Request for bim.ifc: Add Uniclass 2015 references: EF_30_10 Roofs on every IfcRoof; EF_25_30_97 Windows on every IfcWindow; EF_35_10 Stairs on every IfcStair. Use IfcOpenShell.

First a look at what the model holds.

```python
import ifcopenshell

model = ifcopenshell.open("bim.ifc")
print(model.schema)
print("classifications:", [c.Name for c in model.by_type("IfcClassification")])
for ifc_class in ("IfcDoor", "IfcRoof", "IfcStair", "IfcWall", "IfcWindow"):
    print(ifc_class, len(model.by_type(ifc_class)))
```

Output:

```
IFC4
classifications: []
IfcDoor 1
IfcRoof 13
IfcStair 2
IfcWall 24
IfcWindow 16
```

```python
import ifcopenshell
import ifcopenshell.api.classification

model = ifcopenshell.open("bim.ifc")

system = ifcopenshell.api.classification.add_classification(model, classification="Uniclass 2015")

codes = {
    "IfcRoof": ("EF_30_10", "Roofs"),
    "IfcWindow": ("EF_25_30_97", "Windows"),
    "IfcStair": ("EF_35_10", "Stairs"),
}
for ifc_class, (code, name) in codes.items():
    products = model.by_type(ifc_class)
    ifcopenshell.api.classification.add_reference(
        model, products=products, classification=system, identification=code, name=name
    )
    print(code, len(products))

model.write("bim_updated.ifc")
```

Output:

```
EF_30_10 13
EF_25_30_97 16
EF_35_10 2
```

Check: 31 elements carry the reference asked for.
